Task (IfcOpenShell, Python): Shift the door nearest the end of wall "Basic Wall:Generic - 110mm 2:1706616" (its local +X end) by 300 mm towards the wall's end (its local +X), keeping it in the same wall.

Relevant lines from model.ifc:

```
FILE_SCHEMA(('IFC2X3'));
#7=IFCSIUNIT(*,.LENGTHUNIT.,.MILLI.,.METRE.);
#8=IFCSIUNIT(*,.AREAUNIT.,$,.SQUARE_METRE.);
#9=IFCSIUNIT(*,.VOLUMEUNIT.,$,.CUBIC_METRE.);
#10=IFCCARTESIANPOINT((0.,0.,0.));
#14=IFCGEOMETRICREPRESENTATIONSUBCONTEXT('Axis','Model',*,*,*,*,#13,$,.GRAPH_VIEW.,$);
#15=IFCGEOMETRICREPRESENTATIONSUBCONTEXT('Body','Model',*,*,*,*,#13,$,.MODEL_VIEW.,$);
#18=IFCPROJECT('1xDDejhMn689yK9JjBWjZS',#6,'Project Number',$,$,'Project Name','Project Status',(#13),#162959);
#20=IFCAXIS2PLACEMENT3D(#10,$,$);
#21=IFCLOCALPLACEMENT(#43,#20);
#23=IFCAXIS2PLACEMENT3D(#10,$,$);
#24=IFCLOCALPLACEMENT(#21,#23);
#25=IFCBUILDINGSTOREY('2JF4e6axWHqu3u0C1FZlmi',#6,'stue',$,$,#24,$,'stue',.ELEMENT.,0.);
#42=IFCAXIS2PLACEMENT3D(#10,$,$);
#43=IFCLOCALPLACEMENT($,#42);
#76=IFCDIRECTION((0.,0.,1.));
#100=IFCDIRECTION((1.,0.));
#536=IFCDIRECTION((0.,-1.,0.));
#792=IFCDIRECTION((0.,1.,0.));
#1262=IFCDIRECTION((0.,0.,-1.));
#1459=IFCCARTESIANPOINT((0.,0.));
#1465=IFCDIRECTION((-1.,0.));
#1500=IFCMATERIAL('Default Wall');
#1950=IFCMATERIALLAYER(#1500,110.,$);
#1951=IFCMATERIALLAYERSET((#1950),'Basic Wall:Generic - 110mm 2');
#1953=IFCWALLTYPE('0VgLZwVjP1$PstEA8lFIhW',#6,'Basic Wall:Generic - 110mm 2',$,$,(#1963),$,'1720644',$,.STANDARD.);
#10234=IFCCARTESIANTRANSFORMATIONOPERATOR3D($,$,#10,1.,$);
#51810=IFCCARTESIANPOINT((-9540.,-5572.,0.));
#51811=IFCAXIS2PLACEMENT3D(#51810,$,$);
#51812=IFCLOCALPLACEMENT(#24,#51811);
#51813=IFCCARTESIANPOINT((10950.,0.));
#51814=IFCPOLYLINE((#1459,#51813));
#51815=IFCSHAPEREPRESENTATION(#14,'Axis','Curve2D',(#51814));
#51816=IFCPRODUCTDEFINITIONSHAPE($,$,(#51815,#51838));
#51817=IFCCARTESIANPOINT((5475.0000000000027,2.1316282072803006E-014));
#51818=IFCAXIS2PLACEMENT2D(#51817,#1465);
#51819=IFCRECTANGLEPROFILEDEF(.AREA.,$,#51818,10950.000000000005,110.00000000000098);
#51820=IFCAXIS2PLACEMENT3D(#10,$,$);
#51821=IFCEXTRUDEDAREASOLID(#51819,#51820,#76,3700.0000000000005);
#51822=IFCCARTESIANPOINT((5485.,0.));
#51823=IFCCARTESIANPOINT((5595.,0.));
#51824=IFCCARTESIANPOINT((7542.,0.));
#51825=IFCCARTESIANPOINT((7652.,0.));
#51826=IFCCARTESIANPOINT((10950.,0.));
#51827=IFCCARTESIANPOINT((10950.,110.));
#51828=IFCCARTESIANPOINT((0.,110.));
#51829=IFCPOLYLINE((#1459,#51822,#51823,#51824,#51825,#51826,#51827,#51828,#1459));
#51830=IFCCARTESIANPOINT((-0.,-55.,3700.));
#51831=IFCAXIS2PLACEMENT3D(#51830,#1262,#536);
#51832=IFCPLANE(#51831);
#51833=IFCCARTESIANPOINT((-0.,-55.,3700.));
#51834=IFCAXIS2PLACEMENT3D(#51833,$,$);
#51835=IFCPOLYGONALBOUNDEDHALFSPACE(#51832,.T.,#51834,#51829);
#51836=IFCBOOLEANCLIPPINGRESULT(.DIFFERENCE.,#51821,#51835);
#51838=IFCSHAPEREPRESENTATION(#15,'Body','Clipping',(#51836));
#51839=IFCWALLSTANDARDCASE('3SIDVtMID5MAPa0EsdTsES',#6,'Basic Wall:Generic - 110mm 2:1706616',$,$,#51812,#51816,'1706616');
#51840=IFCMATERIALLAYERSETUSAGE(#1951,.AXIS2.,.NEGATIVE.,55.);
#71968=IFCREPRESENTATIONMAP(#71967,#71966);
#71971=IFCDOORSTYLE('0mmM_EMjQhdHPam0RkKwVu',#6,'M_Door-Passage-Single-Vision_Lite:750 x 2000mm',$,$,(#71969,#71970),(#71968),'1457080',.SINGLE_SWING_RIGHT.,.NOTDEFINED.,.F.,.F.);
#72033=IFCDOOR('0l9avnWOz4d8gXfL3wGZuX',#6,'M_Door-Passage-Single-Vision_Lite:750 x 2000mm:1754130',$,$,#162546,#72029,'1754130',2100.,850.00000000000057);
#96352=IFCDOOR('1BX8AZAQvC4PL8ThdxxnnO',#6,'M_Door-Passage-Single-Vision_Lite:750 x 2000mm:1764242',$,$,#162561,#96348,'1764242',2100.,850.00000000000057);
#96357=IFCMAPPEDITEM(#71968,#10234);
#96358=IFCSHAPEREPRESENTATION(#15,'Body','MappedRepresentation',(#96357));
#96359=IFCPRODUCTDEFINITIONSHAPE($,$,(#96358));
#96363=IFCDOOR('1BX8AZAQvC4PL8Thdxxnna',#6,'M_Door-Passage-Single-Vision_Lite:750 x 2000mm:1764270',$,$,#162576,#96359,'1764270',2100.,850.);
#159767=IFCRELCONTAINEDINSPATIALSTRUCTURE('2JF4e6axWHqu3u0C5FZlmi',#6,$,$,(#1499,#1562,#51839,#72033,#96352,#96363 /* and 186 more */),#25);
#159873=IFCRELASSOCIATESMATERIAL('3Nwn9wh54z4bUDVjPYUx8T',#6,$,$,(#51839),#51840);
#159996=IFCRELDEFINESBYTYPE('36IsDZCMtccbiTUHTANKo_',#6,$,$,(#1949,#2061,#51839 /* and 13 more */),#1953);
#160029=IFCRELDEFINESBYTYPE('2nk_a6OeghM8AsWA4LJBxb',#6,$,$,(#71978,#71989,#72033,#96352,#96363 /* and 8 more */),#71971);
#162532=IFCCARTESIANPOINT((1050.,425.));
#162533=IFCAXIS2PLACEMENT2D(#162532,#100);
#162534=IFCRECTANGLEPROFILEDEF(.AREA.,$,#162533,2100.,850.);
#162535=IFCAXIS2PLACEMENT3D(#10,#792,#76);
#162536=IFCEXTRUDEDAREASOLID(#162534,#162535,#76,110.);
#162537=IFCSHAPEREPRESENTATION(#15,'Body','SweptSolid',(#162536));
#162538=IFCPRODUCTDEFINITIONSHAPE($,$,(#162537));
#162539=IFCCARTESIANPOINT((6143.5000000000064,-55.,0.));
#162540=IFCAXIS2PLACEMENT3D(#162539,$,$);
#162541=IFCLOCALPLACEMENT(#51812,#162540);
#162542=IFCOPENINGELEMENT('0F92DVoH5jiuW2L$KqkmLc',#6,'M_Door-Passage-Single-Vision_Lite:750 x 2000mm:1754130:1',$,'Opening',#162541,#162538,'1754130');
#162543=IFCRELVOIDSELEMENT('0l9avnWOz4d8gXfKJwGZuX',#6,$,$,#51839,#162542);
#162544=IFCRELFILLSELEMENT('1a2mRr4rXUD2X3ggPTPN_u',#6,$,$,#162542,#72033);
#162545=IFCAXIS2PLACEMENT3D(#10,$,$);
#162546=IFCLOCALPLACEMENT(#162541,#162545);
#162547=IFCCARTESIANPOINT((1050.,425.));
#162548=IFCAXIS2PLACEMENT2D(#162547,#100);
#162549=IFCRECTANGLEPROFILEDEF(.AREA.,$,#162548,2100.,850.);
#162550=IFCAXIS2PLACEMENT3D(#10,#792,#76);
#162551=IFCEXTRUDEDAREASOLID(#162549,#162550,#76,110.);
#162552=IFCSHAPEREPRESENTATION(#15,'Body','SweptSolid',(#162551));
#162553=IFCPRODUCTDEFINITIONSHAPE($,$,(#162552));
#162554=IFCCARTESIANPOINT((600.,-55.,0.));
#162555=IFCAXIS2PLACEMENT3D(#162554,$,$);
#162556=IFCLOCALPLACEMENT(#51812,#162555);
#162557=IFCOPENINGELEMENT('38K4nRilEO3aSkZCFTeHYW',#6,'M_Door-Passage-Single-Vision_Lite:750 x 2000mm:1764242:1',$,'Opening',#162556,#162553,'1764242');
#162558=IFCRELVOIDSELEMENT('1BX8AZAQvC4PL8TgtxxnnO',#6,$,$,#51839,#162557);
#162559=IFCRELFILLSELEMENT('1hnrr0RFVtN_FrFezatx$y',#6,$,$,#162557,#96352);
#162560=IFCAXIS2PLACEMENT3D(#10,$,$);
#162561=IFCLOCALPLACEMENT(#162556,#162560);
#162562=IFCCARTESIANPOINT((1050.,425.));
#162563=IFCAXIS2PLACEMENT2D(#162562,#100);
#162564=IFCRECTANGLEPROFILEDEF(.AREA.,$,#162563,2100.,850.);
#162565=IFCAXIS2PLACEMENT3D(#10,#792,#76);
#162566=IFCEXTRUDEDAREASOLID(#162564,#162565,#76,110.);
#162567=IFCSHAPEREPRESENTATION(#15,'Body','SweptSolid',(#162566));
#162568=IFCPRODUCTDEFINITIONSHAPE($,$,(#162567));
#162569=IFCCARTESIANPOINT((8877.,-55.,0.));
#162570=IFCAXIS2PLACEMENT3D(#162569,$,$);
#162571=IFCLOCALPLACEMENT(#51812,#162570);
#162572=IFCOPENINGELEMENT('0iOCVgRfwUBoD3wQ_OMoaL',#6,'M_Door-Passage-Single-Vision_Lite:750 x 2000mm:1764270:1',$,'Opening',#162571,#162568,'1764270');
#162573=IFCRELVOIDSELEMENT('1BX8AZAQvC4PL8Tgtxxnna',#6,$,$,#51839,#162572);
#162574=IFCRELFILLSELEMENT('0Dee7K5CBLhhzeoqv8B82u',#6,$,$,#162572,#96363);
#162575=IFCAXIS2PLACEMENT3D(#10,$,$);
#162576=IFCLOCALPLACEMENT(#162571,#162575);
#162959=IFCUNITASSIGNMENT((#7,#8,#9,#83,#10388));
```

```python
import ifcopenshell
import ifcopenshell.api.geometry
import ifcopenshell.util.placement
import ifcopenshell.util.unit

model = ifcopenshell.open("model.ifc")
unit_scale = ifcopenshell.util.unit.calculate_unit_scale(model)

door = model.by_guid("1BX8AZAQvC4PL8Thdxxnna")
opening = door.FillsVoids[0].RelatingOpeningElement
wall = opening.VoidsElements[0].RelatingBuildingElement

wall_matrix = ifcopenshell.util.placement.get_local_placement(wall.ObjectPlacement)
shift = wall_matrix[:3, 0] * 0.3 / unit_scale
before = ifcopenshell.util.placement.get_local_placement(door.ObjectPlacement)[:3, 3].copy()

# The door is placed relative to its opening, so it follows when the opening moves.
matrix = ifcopenshell.util.placement.get_local_placement(opening.ObjectPlacement)
matrix[:3, 3] += shift
ifcopenshell.api.geometry.edit_object_placement(
    model, product=opening, matrix=matrix, is_si=False, should_transform_children=True
)

after = ifcopenshell.util.placement.get_local_placement(door.ObjectPlacement)[:3, 3]
print("door moved by", (after - before).round(3) + 0.0)

model.write("model-out.ifc")
```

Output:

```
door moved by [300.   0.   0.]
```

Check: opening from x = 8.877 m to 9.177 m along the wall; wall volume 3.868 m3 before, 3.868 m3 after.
